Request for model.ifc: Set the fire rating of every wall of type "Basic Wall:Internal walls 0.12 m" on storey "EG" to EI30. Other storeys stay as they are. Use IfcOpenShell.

First a look at what the model holds.

```python
import ifcopenshell
import ifcopenshell.util.element

model = ifcopenshell.open("model.ifc")
print(model.schema)
storey = next(s for s in model.by_type("IfcBuildingStorey") if s.Name == "EG")
walls = [e for e in ifcopenshell.util.element.get_decomposition(storey) if e.is_a("IfcWall")]
seen = {}
for e in walls:
    element_type = ifcopenshell.util.element.get_type(e)
    key = (element_type.Name if element_type != e and element_type else None, ifcopenshell.util.element.get_pset(e, "Pset_WallCommon", "FireRating"))
    seen[key] = seen.get(key, 0) + 1
for (name, value), count in sorted(seen.items(), key=str):
    print(count, "x", name, "|", value)
```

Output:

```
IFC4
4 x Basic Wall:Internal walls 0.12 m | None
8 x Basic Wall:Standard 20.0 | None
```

```python
import ifcopenshell
import ifcopenshell.api.pset
import ifcopenshell.util.element

model = ifcopenshell.open("model.ifc")

storey = next(s for s in model.by_type("IfcBuildingStorey") if s.Name == "EG")
walls = [e for e in ifcopenshell.util.element.get_decomposition(storey) if e.is_a("IfcWall")]

count = 0
for e in walls:
    element_type = ifcopenshell.util.element.get_type(e)
    if element_type in (None, e) or element_type.Name != "Basic Wall:Internal walls 0.12 m":
        continue
    # add_pset returns the element's existing set when there is one.
    pset = ifcopenshell.api.pset.add_pset(model, product=e, name="Pset_WallCommon")
    ifcopenshell.api.pset.edit_pset(model, pset=pset, properties={"FireRating": "EI30"})
    count += 1

print(count, "walls updated")

model.write("model_edited.ifc")
```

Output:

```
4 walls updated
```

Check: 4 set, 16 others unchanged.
